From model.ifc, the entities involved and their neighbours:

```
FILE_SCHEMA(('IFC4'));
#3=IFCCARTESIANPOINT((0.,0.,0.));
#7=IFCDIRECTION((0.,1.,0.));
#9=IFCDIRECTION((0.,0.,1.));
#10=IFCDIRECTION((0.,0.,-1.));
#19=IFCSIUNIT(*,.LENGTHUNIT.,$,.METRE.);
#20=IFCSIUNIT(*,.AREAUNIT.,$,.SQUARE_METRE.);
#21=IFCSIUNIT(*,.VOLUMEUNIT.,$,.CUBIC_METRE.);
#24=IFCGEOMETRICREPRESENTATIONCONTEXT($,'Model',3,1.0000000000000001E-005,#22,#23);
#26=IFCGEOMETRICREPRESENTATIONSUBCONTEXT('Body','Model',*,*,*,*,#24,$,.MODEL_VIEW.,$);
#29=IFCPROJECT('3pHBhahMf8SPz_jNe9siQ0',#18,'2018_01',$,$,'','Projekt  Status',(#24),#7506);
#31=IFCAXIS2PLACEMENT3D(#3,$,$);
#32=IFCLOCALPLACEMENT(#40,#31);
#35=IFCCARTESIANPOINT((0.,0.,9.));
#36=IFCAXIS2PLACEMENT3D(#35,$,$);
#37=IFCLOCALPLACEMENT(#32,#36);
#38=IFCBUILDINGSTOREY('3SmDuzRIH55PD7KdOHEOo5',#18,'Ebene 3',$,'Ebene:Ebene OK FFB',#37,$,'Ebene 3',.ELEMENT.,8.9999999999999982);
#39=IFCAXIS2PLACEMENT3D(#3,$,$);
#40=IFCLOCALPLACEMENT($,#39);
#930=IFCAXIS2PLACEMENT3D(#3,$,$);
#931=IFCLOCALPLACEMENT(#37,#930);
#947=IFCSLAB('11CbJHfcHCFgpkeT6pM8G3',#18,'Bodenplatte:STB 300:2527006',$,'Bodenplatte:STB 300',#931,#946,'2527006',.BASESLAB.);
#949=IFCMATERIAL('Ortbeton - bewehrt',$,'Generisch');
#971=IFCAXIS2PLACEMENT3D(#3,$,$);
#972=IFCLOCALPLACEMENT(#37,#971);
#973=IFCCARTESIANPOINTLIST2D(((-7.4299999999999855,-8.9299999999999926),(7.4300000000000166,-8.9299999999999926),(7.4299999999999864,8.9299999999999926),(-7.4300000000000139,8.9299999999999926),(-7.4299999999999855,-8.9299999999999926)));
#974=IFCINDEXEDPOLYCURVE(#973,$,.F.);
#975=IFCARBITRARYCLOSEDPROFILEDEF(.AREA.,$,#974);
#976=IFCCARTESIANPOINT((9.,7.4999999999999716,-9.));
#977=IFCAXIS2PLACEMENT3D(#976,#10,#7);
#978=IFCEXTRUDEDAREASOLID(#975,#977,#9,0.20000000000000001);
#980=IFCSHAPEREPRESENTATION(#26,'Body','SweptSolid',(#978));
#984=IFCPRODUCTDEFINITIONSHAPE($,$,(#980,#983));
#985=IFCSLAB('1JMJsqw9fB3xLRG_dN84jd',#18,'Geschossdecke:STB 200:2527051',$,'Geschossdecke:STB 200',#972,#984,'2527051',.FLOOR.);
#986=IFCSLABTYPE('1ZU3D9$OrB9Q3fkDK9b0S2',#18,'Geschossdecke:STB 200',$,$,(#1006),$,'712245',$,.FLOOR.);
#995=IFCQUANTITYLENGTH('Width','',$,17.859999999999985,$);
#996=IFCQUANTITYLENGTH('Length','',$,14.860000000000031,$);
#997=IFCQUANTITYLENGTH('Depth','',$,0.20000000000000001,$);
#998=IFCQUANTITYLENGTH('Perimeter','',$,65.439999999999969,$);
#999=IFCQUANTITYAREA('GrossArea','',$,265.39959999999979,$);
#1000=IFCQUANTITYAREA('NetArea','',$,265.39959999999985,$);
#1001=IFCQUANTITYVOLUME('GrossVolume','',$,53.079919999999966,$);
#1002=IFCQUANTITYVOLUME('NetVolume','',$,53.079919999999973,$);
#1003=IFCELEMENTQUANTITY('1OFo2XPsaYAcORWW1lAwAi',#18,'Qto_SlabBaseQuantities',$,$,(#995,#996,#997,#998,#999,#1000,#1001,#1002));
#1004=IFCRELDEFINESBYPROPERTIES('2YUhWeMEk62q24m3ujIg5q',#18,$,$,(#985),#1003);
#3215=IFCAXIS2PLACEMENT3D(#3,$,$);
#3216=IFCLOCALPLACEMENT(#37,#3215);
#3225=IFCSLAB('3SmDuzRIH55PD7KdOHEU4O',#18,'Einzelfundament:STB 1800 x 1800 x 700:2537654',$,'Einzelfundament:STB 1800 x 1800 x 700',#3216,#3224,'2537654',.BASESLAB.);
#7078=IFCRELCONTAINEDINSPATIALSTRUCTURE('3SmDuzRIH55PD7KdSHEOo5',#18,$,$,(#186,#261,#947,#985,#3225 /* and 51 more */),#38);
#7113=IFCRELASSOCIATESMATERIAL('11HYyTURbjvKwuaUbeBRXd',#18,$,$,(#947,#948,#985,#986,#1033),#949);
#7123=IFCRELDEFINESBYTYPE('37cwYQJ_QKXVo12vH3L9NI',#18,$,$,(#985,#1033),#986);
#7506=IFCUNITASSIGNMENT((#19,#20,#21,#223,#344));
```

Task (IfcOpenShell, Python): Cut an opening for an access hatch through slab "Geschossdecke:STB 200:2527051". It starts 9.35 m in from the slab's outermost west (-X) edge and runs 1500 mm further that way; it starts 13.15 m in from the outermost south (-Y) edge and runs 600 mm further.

```python
import numpy as np
import ifcopenshell
import ifcopenshell.api.feature
import ifcopenshell.api.geometry
import ifcopenshell.api.pset
import ifcopenshell.api.root
import ifcopenshell.geom
import ifcopenshell.util.element
import ifcopenshell.util.placement
import ifcopenshell.util.representation
import ifcopenshell.util.shape
import ifcopenshell.util.unit

model = ifcopenshell.open("model.ifc")
unit_scale = ifcopenshell.util.unit.calculate_unit_scale(model)
area_scale = ifcopenshell.util.unit.calculate_unit_scale(model, "AREAUNIT")
volume_scale = ifcopenshell.util.unit.calculate_unit_scale(model, "VOLUMEUNIT")
settings = ifcopenshell.geom.settings()


def volume(element):
    """Net volume in cubic metres, openings subtracted."""
    shape = ifcopenshell.geom.create_shape(settings, element)
    return ifcopenshell.util.shape.get_volume(shape.geometry)


slab = model.by_guid("1JMJsqw9fB3xLRG_dN84jd")
before = volume(slab)

# Extent in the slab's own axes, in metres. The edges named are its -X and -Y sides.
slab_shape = ifcopenshell.geom.create_shape(settings, slab)
vertices = ifcopenshell.util.shape.get_vertices(slab_shape.geometry)
x_min, y_min, bottom = vertices.min(axis=0)
top = vertices[:, 2].max()

opening = ifcopenshell.api.root.create_entity(model, ifc_class="IfcOpeningElement", name="Access hatch opening", predefined_type="OPENING")
context = ifcopenshell.util.representation.get_context(model, "Model", "Body", "MODEL_VIEW")
width, depth = 1.5, 0.6
outline = [(0.0, 0.0), (width, 0.0), (width, depth), (0.0, depth), (0.0, 0.0)]
# Overshoot both faces by 50 mm so the cut is clean.
shape = ifcopenshell.api.geometry.add_slab_representation(
    model, context=context, depth=top - bottom + 0.1, polyline=outline
)
ifcopenshell.api.geometry.assign_representation(model, product=opening, representation=shape)

matrix = ifcopenshell.util.placement.get_local_placement(slab.ObjectPlacement)
matrix[:, 3] = matrix @ np.append(np.array([x_min + 9.35, y_min + 13.15, bottom - 0.05]) / unit_scale, 1.0)
ifcopenshell.api.geometry.edit_object_placement(model, product=opening, matrix=matrix, is_si=False)
ifcopenshell.api.feature.add_feature(model, feature=opening, element=slab)

after = volume(slab)

# Update the slab's stored quantities.
qto = model.by_id(ifcopenshell.util.element.get_pset(slab, "Qto_SlabBaseQuantities", should_inherit=False)["id"])
ifcopenshell.api.pset.edit_qto(model, qto=qto, properties={
    "NetArea": after / (top - bottom) / area_scale,
    "NetVolume": after / volume_scale,
})

print(f"slab volume {before:.3f} -> {after:.3f} m3")

model.write("model_rev.ifc")
```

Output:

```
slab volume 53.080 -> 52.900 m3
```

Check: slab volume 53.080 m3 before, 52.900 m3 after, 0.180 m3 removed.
